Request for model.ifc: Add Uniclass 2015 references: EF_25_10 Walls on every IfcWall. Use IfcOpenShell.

First a look at what the model holds.

```python
import ifcopenshell

model = ifcopenshell.open("model.ifc")
print(model.schema)
print("classifications:", [c.Name for c in model.by_type("IfcClassification")])
for ifc_class in ("IfcDoor", "IfcRoof", "IfcStair", "IfcWall", "IfcWindow"):
    print(ifc_class, len(model.by_type(ifc_class)))
```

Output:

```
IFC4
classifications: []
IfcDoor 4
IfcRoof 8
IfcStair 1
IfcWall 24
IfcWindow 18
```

```python
import ifcopenshell
import ifcopenshell.api.classification

model = ifcopenshell.open("model.ifc")

system = ifcopenshell.api.classification.add_classification(model, classification="Uniclass 2015")

codes = {
    "IfcWall": ("EF_25_10", "Walls"),
}
for ifc_class, (code, name) in codes.items():
    products = model.by_type(ifc_class)
    ifcopenshell.api.classification.add_reference(
        model, products=products, classification=system, identification=code, name=name
    )
    print(code, len(products))

model.write("model_v2.ifc")
```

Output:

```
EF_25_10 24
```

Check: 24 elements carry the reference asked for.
